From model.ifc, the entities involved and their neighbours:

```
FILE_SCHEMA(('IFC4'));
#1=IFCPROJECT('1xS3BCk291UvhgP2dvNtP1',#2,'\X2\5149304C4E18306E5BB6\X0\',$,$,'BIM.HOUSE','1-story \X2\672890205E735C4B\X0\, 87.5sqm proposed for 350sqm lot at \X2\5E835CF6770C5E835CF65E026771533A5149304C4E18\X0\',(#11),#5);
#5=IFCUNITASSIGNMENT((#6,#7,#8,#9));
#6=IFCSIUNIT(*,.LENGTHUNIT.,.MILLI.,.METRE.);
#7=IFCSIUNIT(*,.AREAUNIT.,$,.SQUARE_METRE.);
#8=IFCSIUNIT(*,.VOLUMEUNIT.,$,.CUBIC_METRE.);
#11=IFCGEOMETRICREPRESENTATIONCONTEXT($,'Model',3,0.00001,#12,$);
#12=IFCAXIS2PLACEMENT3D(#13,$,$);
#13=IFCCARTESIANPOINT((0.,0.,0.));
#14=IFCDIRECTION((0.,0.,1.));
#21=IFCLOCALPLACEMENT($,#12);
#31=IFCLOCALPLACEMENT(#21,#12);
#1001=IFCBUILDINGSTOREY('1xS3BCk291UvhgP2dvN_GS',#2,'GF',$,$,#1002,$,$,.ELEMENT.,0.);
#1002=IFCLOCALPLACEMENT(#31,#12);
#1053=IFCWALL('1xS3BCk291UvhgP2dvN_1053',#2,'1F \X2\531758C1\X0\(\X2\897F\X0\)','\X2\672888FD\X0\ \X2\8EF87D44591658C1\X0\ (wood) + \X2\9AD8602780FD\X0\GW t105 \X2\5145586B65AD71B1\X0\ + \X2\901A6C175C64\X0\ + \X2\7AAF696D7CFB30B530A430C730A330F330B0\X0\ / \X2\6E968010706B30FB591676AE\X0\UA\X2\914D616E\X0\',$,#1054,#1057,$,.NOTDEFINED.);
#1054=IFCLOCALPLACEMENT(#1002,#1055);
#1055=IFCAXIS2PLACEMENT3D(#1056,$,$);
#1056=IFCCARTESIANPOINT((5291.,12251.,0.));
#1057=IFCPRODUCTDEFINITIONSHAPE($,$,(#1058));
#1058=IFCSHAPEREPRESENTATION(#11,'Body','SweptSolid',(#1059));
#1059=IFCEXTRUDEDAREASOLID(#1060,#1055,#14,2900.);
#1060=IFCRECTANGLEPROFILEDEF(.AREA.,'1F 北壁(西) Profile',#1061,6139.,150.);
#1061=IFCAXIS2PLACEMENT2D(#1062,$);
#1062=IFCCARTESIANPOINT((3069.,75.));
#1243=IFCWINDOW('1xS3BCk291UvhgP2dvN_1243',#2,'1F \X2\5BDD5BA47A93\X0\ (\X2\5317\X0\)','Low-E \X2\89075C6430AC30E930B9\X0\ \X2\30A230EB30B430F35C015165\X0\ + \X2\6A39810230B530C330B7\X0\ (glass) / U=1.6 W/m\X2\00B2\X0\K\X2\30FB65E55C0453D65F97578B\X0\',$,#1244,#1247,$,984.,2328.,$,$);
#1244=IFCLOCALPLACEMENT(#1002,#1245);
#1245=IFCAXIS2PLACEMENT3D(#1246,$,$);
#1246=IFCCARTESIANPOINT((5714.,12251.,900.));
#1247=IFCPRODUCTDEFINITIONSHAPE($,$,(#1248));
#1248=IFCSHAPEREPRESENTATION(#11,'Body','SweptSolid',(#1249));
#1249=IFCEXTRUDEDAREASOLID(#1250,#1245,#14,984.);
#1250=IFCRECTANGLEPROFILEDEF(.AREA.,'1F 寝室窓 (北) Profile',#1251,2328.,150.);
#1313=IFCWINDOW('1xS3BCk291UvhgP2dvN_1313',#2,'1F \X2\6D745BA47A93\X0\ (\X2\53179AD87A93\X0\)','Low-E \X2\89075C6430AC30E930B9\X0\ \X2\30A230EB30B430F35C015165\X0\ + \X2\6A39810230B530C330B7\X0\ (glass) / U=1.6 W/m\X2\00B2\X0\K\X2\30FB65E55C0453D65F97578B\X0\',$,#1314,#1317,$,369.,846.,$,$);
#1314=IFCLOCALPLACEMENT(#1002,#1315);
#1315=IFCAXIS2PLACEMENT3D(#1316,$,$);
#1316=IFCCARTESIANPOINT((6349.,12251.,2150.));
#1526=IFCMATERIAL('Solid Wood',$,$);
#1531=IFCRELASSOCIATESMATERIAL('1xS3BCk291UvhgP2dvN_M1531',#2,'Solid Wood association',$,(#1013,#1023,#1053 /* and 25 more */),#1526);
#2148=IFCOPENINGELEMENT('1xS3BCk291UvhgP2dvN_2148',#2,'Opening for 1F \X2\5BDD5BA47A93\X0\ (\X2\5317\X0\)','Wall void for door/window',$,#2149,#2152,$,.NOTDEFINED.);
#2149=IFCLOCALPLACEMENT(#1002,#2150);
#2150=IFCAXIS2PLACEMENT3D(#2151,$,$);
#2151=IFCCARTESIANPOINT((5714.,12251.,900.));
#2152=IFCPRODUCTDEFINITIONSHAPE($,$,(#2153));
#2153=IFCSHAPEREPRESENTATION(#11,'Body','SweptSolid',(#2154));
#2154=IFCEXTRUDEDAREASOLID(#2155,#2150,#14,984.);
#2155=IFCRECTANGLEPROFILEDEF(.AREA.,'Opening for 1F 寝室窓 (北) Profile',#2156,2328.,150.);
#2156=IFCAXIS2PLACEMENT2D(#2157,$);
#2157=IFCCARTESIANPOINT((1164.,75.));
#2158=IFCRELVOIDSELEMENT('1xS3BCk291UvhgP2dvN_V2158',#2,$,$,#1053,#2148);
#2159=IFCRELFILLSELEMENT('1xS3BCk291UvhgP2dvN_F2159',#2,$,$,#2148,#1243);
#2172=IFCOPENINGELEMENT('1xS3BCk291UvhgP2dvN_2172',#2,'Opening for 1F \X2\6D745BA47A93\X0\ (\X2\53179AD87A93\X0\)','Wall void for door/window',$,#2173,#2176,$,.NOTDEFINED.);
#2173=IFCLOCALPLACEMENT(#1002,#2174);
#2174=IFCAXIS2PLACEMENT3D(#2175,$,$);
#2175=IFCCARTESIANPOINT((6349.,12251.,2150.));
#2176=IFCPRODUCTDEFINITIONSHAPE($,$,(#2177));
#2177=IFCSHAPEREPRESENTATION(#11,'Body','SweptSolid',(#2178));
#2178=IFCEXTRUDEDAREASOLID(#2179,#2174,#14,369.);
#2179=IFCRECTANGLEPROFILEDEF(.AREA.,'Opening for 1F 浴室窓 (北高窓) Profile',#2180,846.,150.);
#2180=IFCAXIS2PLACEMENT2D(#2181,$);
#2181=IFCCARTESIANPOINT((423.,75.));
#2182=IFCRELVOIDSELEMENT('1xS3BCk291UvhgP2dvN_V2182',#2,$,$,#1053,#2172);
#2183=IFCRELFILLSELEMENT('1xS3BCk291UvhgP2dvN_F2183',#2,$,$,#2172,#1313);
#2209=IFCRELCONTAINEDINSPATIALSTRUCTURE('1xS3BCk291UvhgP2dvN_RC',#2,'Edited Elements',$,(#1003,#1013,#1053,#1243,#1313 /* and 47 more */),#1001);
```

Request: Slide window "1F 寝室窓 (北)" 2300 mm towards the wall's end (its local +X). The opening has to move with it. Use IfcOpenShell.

```python
import ifcopenshell
import ifcopenshell.api.geometry
import ifcopenshell.util.placement

model = ifcopenshell.open("model.ifc")

window = model.by_guid("1xS3BCk291UvhgP2dvN_1243")
opening = window.FillsVoids[0].RelatingOpeningElement
wall = opening.VoidsElements[0].RelatingBuildingElement

wall_matrix = ifcopenshell.util.placement.get_local_placement(wall.ObjectPlacement)
shift = wall_matrix[:3, 0] * 2300.0
before = ifcopenshell.util.placement.get_local_placement(window.ObjectPlacement)[:3, 3].copy()

# The window is not placed relative to its opening, so move both.
for product in (opening, window):
    matrix = ifcopenshell.util.placement.get_local_placement(product.ObjectPlacement)
    matrix[:3, 3] += shift
    ifcopenshell.api.geometry.edit_object_placement(model, product=product, matrix=matrix, is_si=False)

after = ifcopenshell.util.placement.get_local_placement(window.ObjectPlacement)[:3, 3]
print("window moved by", (after - before).round(3) + 0.0)

model.write("model-out.ifc")
```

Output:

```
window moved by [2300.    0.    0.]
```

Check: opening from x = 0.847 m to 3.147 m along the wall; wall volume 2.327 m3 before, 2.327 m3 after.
